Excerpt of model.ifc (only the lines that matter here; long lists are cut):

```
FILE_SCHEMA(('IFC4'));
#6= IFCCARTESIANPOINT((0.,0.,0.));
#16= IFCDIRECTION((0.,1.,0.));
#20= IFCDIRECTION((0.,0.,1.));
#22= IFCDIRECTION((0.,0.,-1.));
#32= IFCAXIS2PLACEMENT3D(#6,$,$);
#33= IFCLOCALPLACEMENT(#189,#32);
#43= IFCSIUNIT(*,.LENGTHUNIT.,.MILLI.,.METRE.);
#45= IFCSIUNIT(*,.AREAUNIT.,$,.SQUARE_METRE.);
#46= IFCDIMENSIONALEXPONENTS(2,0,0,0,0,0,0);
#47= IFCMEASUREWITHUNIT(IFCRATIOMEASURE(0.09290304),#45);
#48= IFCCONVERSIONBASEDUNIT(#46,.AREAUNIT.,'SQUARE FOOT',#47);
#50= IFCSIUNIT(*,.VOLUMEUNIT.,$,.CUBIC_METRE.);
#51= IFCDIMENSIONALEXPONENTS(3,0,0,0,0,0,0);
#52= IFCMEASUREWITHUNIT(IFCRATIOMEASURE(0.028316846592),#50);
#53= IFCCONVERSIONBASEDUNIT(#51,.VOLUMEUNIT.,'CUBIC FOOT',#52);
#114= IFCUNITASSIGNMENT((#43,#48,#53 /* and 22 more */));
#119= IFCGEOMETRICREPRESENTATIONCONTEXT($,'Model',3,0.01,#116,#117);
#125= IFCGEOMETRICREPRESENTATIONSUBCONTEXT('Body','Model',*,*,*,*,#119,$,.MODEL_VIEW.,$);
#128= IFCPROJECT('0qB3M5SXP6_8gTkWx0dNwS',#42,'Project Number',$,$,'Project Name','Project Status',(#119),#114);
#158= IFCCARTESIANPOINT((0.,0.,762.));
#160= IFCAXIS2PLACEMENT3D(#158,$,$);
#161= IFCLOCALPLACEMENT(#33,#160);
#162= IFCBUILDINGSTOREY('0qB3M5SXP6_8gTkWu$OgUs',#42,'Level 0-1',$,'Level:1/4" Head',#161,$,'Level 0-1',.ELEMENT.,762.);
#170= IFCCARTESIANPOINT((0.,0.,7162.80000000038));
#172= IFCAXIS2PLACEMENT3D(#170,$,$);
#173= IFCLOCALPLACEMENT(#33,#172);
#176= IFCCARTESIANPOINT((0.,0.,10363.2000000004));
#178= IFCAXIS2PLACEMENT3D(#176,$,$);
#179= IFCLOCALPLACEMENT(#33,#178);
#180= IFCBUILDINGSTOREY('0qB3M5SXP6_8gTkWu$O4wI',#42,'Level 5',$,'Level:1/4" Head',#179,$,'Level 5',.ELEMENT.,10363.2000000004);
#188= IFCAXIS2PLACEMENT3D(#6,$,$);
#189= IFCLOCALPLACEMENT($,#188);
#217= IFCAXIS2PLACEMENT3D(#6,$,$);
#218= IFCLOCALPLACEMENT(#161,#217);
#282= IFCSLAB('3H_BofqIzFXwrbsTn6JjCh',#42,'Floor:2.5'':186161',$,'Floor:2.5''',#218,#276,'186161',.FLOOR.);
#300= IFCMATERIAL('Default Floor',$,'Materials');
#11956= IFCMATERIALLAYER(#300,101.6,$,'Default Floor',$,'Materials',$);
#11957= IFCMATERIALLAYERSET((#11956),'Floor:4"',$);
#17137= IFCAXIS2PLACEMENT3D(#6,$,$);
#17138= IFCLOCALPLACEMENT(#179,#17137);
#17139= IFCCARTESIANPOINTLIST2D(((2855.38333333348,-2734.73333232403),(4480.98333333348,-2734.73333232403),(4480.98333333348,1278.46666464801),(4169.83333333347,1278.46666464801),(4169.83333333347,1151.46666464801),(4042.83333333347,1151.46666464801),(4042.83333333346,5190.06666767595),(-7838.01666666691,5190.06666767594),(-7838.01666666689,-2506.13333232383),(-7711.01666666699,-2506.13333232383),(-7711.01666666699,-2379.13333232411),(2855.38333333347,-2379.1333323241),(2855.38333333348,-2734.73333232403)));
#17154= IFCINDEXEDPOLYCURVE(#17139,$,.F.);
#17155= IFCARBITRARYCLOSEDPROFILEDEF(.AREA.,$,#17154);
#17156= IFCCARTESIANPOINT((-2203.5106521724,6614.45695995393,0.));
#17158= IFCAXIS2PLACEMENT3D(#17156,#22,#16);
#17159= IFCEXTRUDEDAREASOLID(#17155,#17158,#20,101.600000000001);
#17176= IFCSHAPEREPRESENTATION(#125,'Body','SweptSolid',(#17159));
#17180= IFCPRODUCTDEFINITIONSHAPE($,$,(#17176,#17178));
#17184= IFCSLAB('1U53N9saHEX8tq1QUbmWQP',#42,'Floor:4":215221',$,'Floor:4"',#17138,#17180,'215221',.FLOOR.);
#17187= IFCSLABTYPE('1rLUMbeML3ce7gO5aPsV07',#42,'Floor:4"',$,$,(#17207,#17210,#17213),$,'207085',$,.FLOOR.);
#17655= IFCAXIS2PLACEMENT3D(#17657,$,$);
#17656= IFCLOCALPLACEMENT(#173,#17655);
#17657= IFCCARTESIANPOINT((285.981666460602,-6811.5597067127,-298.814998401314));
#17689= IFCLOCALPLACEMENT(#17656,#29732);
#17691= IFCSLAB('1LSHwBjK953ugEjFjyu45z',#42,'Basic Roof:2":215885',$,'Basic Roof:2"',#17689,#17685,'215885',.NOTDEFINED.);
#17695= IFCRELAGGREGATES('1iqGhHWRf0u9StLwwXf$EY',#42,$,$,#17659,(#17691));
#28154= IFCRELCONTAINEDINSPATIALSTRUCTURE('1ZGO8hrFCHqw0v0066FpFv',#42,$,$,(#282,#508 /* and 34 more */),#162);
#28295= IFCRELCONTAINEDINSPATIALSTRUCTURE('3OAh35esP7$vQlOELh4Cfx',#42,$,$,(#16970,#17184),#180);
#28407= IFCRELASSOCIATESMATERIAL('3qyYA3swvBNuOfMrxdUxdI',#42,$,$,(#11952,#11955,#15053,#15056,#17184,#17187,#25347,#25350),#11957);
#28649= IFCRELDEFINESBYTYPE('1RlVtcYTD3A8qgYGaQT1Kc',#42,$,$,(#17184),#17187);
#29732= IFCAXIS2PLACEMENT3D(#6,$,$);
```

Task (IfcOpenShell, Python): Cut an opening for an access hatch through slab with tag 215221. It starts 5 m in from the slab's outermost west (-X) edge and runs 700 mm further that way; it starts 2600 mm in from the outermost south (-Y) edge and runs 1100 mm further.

```python
import numpy as np
import ifcopenshell
import ifcopenshell.api.feature
import ifcopenshell.api.geometry
import ifcopenshell.api.root
import ifcopenshell.geom
import ifcopenshell.util.placement
import ifcopenshell.util.representation
import ifcopenshell.util.shape
import ifcopenshell.util.unit

model = ifcopenshell.open("model.ifc")
unit_scale = ifcopenshell.util.unit.calculate_unit_scale(model)
settings = ifcopenshell.geom.settings()


def volume(element):
    """Net volume in cubic metres, openings subtracted."""
    shape = ifcopenshell.geom.create_shape(settings, element)
    return ifcopenshell.util.shape.get_volume(shape.geometry)


slab = model.by_id(17184)
before = volume(slab)

# Extent in the slab's own axes, in metres. The edges named are its -X and -Y sides.
slab_shape = ifcopenshell.geom.create_shape(settings, slab)
vertices = ifcopenshell.util.shape.get_vertices(slab_shape.geometry)
x_min, y_min, bottom = vertices.min(axis=0)
top = vertices[:, 2].max()

opening = ifcopenshell.api.root.create_entity(model, ifc_class="IfcOpeningElement", name="Access hatch opening", predefined_type="OPENING")
context = ifcopenshell.util.representation.get_context(model, "Model", "Body", "MODEL_VIEW")
width, depth = 0.7, 1.1
outline = [(0.0, 0.0), (width, 0.0), (width, depth), (0.0, depth), (0.0, 0.0)]
# Overshoot both faces by 50 mm so the cut is clean.
shape = ifcopenshell.api.geometry.add_slab_representation(
    model, context=context, depth=top - bottom + 0.1, polyline=outline
)
ifcopenshell.api.geometry.assign_representation(model, product=opening, representation=shape)

matrix = ifcopenshell.util.placement.get_local_placement(slab.ObjectPlacement)
matrix[:, 3] = matrix @ np.append(np.array([x_min + 5, y_min + 2.6, bottom - 0.05]) / unit_scale, 1.0)
ifcopenshell.api.geometry.edit_object_placement(model, product=opening, matrix=matrix, is_si=False)
ifcopenshell.api.feature.add_feature(model, feature=opening, element=slab)

after = volume(slab)

print(f"slab volume {before:.3f} -> {after:.3f} m3")

model.write("model_v2.ifc")
```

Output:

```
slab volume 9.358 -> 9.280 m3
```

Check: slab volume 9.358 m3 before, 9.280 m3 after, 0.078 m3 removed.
